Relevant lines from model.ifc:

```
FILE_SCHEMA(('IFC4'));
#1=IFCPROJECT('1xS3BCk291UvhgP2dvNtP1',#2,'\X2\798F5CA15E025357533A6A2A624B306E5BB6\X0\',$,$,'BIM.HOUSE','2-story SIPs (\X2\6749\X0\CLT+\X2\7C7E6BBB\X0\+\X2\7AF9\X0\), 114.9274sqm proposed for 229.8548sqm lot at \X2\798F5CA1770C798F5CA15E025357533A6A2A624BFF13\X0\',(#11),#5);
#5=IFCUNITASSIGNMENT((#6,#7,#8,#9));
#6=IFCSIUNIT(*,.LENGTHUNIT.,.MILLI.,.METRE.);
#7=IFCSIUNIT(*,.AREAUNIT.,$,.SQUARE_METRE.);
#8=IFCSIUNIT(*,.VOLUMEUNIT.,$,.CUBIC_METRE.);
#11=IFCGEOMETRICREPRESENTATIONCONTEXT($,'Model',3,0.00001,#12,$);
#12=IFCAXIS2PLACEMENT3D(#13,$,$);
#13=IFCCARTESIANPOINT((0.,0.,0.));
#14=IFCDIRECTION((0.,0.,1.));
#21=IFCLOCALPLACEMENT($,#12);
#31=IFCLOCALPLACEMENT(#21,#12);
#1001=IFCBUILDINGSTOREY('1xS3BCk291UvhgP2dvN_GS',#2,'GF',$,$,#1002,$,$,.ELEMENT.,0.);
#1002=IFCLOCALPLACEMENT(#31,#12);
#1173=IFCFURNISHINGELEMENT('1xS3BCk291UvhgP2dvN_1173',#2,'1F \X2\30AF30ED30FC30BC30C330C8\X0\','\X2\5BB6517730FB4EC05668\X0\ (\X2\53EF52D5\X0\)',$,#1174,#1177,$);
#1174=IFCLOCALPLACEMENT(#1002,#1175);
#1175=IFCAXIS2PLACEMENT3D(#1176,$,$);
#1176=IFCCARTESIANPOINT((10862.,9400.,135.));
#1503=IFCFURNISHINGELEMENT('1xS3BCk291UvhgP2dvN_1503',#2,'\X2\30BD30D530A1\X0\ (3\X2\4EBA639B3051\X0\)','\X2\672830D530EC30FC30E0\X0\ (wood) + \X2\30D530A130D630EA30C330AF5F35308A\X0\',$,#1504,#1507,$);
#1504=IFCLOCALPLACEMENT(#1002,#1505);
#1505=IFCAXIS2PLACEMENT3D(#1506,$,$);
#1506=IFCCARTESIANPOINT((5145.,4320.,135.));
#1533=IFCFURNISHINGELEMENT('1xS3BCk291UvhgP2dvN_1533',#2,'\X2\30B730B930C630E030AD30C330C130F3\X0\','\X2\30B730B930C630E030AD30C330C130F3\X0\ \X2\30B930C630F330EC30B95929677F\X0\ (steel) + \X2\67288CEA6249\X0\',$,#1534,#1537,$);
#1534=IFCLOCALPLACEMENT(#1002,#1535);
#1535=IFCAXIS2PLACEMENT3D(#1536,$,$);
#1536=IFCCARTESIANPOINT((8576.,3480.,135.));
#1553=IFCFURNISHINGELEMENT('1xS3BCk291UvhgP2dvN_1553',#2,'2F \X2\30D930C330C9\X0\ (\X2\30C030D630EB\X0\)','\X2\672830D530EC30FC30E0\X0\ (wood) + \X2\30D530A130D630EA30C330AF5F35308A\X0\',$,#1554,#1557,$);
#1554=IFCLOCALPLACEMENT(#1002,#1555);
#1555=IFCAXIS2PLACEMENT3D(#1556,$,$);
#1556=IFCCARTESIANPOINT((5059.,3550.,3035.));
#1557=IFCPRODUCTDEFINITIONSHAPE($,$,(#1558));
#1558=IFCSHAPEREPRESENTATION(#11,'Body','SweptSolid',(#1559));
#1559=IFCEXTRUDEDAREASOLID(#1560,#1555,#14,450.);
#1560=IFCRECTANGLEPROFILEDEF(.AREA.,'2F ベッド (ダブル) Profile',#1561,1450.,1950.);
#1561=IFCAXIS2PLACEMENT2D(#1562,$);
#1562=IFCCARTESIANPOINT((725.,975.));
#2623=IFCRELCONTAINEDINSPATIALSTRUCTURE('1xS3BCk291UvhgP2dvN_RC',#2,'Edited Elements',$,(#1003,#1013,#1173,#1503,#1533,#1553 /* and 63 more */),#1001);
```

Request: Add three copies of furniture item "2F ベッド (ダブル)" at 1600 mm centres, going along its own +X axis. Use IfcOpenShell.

```python
import ifcopenshell
import ifcopenshell.api.geometry
import ifcopenshell.api.root
import ifcopenshell.util.element
import ifcopenshell.util.placement
import ifcopenshell.util.unit

model = ifcopenshell.open("model.ifc")
unit_scale = ifcopenshell.util.unit.calculate_unit_scale(model)


def reuse_history(source, copy):
    """copy_class also copies each property set's owner history, people and application; keep the originals."""
    for rel in copy.IsDefinedBy:
        if rel.is_a("IfcRelDefinesByProperties") and (history := rel.RelatingPropertyDefinition.OwnerHistory):
            rel.RelatingPropertyDefinition.OwnerHistory = source.OwnerHistory
            ifcopenshell.util.element.remove_deep2(model, history)


source = model.by_guid("1xS3BCk291UvhgP2dvN_1553")
base = ifcopenshell.util.placement.get_local_placement(source.ObjectPlacement)
step = base[:3, 0] * 1.6 / unit_scale

for i in range(1, 4):
    copy = ifcopenshell.api.root.copy_class(model, product=source)
    copy.Representation = ifcopenshell.util.element.copy_deep(
        model, source.Representation, exclude=["IfcGeometricRepresentationContext", "IfcRepresentationMap"]
    )
    reuse_history(source, copy)
    matrix = base.copy()
    matrix[:3, 3] += i * step
    print("added at", matrix[:3, 3].round(3) + 0.0)
    ifcopenshell.api.geometry.edit_object_placement(model, product=copy, matrix=matrix, is_si=False)

model.write("model-out.ifc")
```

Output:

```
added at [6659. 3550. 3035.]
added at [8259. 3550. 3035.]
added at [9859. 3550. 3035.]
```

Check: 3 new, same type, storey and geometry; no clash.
